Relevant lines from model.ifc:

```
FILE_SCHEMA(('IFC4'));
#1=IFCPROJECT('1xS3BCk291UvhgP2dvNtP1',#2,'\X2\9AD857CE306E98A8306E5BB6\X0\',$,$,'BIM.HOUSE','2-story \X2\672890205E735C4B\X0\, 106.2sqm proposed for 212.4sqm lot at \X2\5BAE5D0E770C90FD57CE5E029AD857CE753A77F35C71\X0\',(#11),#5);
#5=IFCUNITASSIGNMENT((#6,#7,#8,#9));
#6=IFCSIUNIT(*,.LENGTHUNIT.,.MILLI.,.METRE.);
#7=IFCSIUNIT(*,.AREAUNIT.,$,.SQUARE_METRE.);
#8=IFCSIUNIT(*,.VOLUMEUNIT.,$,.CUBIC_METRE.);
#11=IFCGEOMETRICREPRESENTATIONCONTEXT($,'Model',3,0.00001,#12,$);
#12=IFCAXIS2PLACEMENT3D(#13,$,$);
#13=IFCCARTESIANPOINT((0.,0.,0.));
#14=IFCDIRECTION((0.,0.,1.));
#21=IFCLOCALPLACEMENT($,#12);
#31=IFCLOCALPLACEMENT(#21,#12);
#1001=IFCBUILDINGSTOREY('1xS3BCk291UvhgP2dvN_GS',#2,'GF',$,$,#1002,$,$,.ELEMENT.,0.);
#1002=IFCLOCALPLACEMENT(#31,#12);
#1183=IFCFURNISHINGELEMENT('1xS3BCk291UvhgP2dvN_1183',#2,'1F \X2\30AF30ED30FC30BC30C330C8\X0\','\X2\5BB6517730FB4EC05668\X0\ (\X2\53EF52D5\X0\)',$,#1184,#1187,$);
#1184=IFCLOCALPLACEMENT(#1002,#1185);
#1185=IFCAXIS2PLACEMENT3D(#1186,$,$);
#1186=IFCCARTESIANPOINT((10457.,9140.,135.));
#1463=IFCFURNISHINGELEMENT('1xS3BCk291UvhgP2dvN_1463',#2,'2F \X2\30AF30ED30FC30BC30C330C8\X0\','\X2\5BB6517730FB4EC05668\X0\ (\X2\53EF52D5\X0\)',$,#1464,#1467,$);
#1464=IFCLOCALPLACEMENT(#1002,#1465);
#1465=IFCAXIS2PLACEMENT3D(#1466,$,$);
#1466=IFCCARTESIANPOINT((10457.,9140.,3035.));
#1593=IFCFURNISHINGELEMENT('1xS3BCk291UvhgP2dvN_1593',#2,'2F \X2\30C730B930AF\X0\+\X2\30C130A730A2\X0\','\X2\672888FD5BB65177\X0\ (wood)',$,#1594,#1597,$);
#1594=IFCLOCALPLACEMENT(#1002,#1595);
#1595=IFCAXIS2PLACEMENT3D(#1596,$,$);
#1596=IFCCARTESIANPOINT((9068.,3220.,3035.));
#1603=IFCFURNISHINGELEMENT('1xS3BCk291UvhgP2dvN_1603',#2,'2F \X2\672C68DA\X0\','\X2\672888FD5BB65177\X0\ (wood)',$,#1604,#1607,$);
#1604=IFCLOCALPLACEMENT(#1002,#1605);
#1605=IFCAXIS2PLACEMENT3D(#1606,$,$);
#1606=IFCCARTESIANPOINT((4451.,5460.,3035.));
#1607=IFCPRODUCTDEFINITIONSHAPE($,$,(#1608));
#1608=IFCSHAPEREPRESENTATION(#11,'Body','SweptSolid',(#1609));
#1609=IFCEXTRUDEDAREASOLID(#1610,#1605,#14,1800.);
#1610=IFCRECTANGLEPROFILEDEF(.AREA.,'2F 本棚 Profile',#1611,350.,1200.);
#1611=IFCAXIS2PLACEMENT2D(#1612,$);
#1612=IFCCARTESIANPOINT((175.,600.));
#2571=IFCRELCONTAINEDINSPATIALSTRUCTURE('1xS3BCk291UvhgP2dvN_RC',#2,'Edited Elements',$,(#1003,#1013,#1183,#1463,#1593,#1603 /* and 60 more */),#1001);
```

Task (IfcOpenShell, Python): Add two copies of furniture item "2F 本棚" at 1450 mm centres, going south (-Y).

```python
import numpy as np
import ifcopenshell
import ifcopenshell.api.geometry
import ifcopenshell.api.root
import ifcopenshell.util.element
import ifcopenshell.util.placement

model = ifcopenshell.open("model.ifc")


def reuse_history(source, copy):
    """copy_class also copies each property set's owner history, people and application; keep the originals."""
    for rel in copy.IsDefinedBy:
        if rel.is_a("IfcRelDefinesByProperties") and (history := rel.RelatingPropertyDefinition.OwnerHistory):
            rel.RelatingPropertyDefinition.OwnerHistory = source.OwnerHistory
            ifcopenshell.util.element.remove_deep2(model, history)


source = model.by_guid("1xS3BCk291UvhgP2dvN_1603")
base = ifcopenshell.util.placement.get_local_placement(source.ObjectPlacement)
step = np.array([0.0, -1.0, 0.0]) * 1450.0

for i in range(1, 3):
    copy = ifcopenshell.api.root.copy_class(model, product=source)
    copy.Representation = ifcopenshell.util.element.copy_deep(
        model, source.Representation, exclude=["IfcGeometricRepresentationContext", "IfcRepresentationMap"]
    )
    reuse_history(source, copy)
    matrix = base.copy()
    matrix[:3, 3] += i * step
    print("added at", matrix[:3, 3].round(3) + 0.0)
    ifcopenshell.api.geometry.edit_object_placement(model, product=copy, matrix=matrix, is_si=False)

model.write("model_edited.ifc")
```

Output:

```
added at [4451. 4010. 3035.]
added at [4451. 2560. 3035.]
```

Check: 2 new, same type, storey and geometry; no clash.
